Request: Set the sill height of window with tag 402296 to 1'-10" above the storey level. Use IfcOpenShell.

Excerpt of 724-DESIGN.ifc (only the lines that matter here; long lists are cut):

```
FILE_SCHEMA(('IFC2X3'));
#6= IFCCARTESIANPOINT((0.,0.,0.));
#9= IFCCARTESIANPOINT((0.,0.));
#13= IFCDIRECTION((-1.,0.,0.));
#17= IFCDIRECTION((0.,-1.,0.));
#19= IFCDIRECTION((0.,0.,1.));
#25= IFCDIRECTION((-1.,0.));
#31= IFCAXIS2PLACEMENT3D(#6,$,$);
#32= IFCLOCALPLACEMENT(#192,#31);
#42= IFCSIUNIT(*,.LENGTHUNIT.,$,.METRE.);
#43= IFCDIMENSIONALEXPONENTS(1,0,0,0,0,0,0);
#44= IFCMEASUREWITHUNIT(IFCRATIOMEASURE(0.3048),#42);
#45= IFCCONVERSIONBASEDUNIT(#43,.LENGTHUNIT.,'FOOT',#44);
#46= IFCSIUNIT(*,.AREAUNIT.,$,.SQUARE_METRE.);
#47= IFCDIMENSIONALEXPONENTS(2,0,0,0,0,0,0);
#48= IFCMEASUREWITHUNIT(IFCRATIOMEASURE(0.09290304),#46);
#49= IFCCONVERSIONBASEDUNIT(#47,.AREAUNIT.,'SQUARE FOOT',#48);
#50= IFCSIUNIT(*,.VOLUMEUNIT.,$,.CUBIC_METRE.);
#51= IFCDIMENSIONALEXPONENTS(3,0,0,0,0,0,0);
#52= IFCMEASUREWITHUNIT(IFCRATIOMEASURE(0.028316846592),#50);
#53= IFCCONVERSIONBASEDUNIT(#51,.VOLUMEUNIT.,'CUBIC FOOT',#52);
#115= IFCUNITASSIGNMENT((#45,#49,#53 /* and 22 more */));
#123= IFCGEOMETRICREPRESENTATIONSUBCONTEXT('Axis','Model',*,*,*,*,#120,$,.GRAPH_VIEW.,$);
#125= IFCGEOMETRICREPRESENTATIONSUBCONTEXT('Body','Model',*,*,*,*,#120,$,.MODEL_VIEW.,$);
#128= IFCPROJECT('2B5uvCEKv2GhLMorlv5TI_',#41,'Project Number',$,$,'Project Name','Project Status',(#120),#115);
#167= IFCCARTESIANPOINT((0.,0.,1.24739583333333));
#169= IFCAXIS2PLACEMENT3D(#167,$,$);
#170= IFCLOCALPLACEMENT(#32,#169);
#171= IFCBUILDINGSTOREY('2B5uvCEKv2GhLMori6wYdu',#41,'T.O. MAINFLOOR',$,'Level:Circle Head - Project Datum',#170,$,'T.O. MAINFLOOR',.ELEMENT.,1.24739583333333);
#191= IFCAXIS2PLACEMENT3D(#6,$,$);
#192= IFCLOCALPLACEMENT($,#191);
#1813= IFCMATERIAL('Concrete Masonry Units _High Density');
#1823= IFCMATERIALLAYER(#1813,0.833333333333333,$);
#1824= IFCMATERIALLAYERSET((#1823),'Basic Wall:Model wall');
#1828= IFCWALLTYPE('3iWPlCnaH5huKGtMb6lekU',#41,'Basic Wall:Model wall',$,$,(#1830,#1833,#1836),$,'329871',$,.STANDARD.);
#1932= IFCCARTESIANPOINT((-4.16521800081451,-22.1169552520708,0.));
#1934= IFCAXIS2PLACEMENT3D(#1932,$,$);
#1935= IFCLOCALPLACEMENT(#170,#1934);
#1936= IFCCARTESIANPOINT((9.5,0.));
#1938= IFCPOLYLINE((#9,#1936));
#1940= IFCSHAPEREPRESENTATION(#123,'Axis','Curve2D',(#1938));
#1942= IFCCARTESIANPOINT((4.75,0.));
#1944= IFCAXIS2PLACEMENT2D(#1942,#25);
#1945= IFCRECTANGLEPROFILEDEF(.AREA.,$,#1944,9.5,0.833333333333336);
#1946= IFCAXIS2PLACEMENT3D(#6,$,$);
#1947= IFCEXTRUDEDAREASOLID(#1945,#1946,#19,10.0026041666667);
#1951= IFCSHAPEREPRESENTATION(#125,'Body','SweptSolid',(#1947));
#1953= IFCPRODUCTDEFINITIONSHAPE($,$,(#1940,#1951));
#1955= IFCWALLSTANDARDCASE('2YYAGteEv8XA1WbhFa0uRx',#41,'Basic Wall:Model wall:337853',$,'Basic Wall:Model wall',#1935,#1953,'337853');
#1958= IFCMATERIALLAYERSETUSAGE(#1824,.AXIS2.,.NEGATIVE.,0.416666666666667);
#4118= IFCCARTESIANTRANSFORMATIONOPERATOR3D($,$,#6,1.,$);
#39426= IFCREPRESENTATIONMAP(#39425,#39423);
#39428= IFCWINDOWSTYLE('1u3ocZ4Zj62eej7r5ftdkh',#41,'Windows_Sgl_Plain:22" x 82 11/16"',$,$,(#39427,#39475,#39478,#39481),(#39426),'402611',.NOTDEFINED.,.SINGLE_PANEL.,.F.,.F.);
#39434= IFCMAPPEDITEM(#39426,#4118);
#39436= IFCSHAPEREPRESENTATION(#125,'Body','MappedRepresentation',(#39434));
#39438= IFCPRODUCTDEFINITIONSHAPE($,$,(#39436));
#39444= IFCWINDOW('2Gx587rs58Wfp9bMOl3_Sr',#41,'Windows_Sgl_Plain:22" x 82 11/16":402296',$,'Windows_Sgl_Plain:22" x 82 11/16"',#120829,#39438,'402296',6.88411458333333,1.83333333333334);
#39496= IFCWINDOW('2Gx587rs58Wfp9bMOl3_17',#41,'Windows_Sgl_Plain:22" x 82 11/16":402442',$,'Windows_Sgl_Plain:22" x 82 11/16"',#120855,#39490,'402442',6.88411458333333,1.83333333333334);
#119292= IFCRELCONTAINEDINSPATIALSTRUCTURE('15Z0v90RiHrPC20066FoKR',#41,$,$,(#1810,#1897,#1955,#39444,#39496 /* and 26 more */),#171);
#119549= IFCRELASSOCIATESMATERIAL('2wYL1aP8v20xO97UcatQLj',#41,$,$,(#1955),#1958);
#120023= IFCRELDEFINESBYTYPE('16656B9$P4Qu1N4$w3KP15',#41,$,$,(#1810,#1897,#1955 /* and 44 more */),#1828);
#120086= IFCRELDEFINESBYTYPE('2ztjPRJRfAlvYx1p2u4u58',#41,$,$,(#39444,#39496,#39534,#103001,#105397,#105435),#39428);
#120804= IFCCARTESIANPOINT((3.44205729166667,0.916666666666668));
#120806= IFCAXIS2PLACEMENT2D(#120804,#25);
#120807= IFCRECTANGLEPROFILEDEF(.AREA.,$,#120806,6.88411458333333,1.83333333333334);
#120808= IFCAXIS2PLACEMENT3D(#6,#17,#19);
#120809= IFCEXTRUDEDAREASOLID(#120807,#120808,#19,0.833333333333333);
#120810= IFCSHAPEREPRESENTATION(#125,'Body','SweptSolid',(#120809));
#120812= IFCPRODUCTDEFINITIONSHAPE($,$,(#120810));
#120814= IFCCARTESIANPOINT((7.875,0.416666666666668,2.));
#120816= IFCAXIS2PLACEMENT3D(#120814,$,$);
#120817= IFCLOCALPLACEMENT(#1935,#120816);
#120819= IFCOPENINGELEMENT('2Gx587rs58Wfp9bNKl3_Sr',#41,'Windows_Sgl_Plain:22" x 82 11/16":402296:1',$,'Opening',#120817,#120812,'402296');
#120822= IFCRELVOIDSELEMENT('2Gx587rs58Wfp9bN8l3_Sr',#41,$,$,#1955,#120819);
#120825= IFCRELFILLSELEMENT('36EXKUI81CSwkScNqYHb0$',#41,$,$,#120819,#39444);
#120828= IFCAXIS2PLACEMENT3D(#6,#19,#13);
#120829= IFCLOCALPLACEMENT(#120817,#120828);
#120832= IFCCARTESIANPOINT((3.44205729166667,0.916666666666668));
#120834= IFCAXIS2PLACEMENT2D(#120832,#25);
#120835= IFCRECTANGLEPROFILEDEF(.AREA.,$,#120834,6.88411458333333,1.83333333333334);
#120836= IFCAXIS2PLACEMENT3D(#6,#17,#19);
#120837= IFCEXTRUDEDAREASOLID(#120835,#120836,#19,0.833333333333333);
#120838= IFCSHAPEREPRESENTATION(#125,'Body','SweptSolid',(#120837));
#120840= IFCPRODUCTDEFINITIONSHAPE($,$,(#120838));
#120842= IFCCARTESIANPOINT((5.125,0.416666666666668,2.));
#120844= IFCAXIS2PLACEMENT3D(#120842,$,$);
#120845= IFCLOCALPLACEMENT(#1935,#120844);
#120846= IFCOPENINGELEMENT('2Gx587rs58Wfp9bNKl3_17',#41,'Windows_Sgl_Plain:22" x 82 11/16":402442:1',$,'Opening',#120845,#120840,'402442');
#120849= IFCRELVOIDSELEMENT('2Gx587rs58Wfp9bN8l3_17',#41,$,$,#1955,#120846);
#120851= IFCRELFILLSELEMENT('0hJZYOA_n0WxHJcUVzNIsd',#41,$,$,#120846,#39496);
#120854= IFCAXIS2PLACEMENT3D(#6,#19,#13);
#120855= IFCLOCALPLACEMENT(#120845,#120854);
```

```python
import numpy as np
import ifcopenshell
import ifcopenshell.api.geometry
import ifcopenshell.geom
import ifcopenshell.util.element
import ifcopenshell.util.placement
import ifcopenshell.util.shape
import ifcopenshell.util.unit

model = ifcopenshell.open("724-DESIGN.ifc")
unit_scale = ifcopenshell.util.unit.calculate_unit_scale(model)

window = model.by_id(39444)
opening = window.FillsVoids[0].RelatingOpeningElement
storey = ifcopenshell.util.element.get_container(window, ifc_class="IfcBuildingStorey")
level = ifcopenshell.util.placement.get_local_placement(storey.ObjectPlacement)[2, 3]

# The opening's origin need not be at the sill, so measure its lowest point.
shape = ifcopenshell.geom.create_shape(ifcopenshell.geom.settings(), opening)
bottom = ifcopenshell.util.shape.get_shape_bottom_elevation(shape, shape.geometry) / unit_scale
dz = level + 22 * 0.0254 / unit_scale - bottom

shift = np.array([0.0, 0.0, dz])
# The window is placed relative to its opening, so it follows when the opening moves.
matrix = ifcopenshell.util.placement.get_local_placement(opening.ObjectPlacement)
matrix[:3, 3] += shift
ifcopenshell.api.geometry.edit_object_placement(
    model, product=opening, matrix=matrix, is_si=False, should_transform_children=True
)

print(f"moved by {dz * unit_scale:+.3f} m")

model.write("724-DESIGN-out.ifc")
```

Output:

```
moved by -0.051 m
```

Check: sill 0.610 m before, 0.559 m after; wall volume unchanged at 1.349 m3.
